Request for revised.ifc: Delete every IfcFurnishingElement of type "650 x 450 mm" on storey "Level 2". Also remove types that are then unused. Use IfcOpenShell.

First a look at what the model holds.

```python
import ifcopenshell
import ifcopenshell.util.element

model = ifcopenshell.open("revised.ifc")
print(model.schema)
storey = next(s for s in model.by_type("IfcBuildingStorey") if s.Name == "Level 2")
furniture = [e for e in ifcopenshell.util.element.get_decomposition(storey) if e.is_a("IfcFurnishingElement")]
seen = {}
for e in furniture:
    element_type = ifcopenshell.util.element.get_type(e)
    name = element_type.Name if element_type not in (None, e) else None
    seen[name] = seen.get(name, 0) + 1
for name, count in sorted(seen.items(), key=str):
    print(count, "x", name)
```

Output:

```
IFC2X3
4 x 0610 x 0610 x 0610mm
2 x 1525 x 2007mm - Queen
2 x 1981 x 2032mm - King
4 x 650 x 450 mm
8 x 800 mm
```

```python
import ifcopenshell
import ifcopenshell.api.root
import ifcopenshell.util.element

model = ifcopenshell.open("revised.ifc")

storey = next(s for s in model.by_type("IfcBuildingStorey") if s.Name == "Level 2")
furniture = [e for e in ifcopenshell.util.element.get_decomposition(storey) if e.is_a("IfcFurnishingElement")]
targets = [e for e in furniture if (t := ifcopenshell.util.element.get_type(e)) not in (None, e) and t.Name == "650 x 450 mm"]
types = {ifcopenshell.util.element.get_type(e) for e in targets} - {None, *targets}

for e in targets:
    ifcopenshell.api.root.remove_product(model, product=e)
print(len(targets), "removed")

unused = [t for t in types if not ifcopenshell.util.element.get_types(t)]
for t in unused:
    ifcopenshell.api.root.remove_product(model, product=t)
print(len(unused), "unused types removed")

model.write("revised_updated.ifc")
```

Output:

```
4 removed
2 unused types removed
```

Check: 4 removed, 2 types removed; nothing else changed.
